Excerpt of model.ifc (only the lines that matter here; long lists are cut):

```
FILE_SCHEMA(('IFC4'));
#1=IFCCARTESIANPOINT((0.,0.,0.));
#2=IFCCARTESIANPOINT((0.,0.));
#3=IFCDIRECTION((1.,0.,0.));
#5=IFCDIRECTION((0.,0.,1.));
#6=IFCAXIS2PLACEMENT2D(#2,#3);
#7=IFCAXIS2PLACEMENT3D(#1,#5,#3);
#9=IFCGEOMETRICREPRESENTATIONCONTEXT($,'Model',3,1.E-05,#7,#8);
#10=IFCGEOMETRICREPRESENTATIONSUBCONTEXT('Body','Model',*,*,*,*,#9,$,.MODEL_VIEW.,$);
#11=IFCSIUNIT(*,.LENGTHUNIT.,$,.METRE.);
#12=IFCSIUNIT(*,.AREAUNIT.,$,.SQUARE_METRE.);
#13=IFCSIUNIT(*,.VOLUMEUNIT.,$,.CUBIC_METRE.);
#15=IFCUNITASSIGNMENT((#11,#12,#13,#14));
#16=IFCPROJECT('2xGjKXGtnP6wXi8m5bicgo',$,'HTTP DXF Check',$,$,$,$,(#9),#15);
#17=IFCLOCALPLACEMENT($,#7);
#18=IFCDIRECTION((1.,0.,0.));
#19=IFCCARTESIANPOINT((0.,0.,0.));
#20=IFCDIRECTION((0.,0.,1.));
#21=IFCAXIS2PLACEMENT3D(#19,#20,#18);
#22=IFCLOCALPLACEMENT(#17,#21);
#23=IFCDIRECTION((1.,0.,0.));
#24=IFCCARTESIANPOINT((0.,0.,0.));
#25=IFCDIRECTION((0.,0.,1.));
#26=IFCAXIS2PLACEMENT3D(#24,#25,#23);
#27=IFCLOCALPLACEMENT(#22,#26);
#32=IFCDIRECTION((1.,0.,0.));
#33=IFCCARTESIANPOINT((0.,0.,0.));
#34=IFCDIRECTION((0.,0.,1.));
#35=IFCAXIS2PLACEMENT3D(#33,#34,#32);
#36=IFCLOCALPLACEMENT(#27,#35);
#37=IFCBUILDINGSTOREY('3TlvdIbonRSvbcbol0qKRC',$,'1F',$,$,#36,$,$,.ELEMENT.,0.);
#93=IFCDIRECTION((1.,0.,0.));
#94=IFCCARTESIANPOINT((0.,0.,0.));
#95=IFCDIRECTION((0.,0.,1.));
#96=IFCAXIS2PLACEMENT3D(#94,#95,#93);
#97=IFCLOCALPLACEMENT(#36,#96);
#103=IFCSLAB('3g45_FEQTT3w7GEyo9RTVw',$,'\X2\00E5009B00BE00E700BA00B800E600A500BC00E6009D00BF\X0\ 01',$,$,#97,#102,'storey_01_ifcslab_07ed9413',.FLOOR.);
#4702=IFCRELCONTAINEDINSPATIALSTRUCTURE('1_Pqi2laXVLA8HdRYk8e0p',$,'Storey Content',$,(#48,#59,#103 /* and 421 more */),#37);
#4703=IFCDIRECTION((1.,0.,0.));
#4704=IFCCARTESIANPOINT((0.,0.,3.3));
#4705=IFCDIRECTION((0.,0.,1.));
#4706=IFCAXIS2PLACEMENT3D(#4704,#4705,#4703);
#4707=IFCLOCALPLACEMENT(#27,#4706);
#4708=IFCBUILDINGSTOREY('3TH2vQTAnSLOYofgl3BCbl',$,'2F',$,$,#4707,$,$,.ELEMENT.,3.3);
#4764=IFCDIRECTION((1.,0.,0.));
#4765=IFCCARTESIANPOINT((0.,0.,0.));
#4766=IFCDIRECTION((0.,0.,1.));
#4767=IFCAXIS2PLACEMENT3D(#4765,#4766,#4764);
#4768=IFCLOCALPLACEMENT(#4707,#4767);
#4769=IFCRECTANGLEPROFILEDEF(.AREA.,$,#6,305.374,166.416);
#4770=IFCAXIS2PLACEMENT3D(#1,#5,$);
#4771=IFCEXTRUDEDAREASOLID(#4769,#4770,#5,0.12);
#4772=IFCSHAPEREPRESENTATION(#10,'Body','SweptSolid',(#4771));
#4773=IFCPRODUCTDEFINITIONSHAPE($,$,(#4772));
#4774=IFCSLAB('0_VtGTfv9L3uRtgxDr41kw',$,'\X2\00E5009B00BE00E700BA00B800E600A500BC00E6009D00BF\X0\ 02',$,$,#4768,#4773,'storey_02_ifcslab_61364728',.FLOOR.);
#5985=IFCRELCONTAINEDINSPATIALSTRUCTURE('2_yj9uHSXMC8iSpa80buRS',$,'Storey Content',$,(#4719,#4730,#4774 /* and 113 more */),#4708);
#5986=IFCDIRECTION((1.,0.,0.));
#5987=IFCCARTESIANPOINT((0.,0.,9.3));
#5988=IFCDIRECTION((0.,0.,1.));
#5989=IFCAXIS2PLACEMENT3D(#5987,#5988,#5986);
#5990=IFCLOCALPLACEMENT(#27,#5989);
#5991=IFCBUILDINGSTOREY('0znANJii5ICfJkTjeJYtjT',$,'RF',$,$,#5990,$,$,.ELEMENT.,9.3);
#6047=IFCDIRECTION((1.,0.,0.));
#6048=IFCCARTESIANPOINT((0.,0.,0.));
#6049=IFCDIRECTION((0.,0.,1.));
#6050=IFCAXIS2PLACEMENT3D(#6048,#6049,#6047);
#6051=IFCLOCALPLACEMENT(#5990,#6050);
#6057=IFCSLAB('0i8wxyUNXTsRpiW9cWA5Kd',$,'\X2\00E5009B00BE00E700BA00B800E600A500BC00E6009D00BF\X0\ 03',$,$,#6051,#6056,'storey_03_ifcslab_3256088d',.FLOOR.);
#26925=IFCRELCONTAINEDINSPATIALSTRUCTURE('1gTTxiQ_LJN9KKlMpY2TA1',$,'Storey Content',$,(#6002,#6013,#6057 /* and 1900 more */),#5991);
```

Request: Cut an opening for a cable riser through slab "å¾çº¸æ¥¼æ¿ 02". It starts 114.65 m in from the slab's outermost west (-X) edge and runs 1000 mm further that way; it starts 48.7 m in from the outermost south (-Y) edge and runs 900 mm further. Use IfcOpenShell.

```python
import numpy as np
import ifcopenshell
import ifcopenshell.api.feature
import ifcopenshell.api.geometry
import ifcopenshell.api.root
import ifcopenshell.geom
import ifcopenshell.util.placement
import ifcopenshell.util.representation
import ifcopenshell.util.shape
import ifcopenshell.util.unit

model = ifcopenshell.open("model.ifc")
unit_scale = ifcopenshell.util.unit.calculate_unit_scale(model)
settings = ifcopenshell.geom.settings()


def volume(element):
    """Net volume in cubic metres, openings subtracted."""
    shape = ifcopenshell.geom.create_shape(settings, element)
    return ifcopenshell.util.shape.get_volume(shape.geometry)


slab = model.by_guid("0_VtGTfv9L3uRtgxDr41kw")
before = volume(slab)

# Extent in the slab's own axes, in metres. The edges named are its -X and -Y sides.
slab_shape = ifcopenshell.geom.create_shape(settings, slab)
vertices = ifcopenshell.util.shape.get_vertices(slab_shape.geometry)
x_min, y_min, bottom = vertices.min(axis=0)
top = vertices[:, 2].max()

opening = ifcopenshell.api.root.create_entity(model, ifc_class="IfcOpeningElement", name="Cable riser opening", predefined_type="OPENING")
context = ifcopenshell.util.representation.get_context(model, "Model", "Body", "MODEL_VIEW")
width, depth = 1, 0.9
outline = [(0.0, 0.0), (width, 0.0), (width, depth), (0.0, depth), (0.0, 0.0)]
# Overshoot both faces by 50 mm so the cut is clean.
shape = ifcopenshell.api.geometry.add_slab_representation(
    model, context=context, depth=top - bottom + 0.1, polyline=outline
)
ifcopenshell.api.geometry.assign_representation(model, product=opening, representation=shape)

matrix = ifcopenshell.util.placement.get_local_placement(slab.ObjectPlacement)
matrix[:, 3] = matrix @ np.append(np.array([x_min + 114.65, y_min + 48.7, bottom - 0.05]) / unit_scale, 1.0)
ifcopenshell.api.geometry.edit_object_placement(model, product=opening, matrix=matrix, is_si=False)
ifcopenshell.api.feature.add_feature(model, feature=opening, element=slab)

after = volume(slab)

print(f"slab volume {before:.3f} -> {after:.3f} m3")

model.write("model-out.ifc")
```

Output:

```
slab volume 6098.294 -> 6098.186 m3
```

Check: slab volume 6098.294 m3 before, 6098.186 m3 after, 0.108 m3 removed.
